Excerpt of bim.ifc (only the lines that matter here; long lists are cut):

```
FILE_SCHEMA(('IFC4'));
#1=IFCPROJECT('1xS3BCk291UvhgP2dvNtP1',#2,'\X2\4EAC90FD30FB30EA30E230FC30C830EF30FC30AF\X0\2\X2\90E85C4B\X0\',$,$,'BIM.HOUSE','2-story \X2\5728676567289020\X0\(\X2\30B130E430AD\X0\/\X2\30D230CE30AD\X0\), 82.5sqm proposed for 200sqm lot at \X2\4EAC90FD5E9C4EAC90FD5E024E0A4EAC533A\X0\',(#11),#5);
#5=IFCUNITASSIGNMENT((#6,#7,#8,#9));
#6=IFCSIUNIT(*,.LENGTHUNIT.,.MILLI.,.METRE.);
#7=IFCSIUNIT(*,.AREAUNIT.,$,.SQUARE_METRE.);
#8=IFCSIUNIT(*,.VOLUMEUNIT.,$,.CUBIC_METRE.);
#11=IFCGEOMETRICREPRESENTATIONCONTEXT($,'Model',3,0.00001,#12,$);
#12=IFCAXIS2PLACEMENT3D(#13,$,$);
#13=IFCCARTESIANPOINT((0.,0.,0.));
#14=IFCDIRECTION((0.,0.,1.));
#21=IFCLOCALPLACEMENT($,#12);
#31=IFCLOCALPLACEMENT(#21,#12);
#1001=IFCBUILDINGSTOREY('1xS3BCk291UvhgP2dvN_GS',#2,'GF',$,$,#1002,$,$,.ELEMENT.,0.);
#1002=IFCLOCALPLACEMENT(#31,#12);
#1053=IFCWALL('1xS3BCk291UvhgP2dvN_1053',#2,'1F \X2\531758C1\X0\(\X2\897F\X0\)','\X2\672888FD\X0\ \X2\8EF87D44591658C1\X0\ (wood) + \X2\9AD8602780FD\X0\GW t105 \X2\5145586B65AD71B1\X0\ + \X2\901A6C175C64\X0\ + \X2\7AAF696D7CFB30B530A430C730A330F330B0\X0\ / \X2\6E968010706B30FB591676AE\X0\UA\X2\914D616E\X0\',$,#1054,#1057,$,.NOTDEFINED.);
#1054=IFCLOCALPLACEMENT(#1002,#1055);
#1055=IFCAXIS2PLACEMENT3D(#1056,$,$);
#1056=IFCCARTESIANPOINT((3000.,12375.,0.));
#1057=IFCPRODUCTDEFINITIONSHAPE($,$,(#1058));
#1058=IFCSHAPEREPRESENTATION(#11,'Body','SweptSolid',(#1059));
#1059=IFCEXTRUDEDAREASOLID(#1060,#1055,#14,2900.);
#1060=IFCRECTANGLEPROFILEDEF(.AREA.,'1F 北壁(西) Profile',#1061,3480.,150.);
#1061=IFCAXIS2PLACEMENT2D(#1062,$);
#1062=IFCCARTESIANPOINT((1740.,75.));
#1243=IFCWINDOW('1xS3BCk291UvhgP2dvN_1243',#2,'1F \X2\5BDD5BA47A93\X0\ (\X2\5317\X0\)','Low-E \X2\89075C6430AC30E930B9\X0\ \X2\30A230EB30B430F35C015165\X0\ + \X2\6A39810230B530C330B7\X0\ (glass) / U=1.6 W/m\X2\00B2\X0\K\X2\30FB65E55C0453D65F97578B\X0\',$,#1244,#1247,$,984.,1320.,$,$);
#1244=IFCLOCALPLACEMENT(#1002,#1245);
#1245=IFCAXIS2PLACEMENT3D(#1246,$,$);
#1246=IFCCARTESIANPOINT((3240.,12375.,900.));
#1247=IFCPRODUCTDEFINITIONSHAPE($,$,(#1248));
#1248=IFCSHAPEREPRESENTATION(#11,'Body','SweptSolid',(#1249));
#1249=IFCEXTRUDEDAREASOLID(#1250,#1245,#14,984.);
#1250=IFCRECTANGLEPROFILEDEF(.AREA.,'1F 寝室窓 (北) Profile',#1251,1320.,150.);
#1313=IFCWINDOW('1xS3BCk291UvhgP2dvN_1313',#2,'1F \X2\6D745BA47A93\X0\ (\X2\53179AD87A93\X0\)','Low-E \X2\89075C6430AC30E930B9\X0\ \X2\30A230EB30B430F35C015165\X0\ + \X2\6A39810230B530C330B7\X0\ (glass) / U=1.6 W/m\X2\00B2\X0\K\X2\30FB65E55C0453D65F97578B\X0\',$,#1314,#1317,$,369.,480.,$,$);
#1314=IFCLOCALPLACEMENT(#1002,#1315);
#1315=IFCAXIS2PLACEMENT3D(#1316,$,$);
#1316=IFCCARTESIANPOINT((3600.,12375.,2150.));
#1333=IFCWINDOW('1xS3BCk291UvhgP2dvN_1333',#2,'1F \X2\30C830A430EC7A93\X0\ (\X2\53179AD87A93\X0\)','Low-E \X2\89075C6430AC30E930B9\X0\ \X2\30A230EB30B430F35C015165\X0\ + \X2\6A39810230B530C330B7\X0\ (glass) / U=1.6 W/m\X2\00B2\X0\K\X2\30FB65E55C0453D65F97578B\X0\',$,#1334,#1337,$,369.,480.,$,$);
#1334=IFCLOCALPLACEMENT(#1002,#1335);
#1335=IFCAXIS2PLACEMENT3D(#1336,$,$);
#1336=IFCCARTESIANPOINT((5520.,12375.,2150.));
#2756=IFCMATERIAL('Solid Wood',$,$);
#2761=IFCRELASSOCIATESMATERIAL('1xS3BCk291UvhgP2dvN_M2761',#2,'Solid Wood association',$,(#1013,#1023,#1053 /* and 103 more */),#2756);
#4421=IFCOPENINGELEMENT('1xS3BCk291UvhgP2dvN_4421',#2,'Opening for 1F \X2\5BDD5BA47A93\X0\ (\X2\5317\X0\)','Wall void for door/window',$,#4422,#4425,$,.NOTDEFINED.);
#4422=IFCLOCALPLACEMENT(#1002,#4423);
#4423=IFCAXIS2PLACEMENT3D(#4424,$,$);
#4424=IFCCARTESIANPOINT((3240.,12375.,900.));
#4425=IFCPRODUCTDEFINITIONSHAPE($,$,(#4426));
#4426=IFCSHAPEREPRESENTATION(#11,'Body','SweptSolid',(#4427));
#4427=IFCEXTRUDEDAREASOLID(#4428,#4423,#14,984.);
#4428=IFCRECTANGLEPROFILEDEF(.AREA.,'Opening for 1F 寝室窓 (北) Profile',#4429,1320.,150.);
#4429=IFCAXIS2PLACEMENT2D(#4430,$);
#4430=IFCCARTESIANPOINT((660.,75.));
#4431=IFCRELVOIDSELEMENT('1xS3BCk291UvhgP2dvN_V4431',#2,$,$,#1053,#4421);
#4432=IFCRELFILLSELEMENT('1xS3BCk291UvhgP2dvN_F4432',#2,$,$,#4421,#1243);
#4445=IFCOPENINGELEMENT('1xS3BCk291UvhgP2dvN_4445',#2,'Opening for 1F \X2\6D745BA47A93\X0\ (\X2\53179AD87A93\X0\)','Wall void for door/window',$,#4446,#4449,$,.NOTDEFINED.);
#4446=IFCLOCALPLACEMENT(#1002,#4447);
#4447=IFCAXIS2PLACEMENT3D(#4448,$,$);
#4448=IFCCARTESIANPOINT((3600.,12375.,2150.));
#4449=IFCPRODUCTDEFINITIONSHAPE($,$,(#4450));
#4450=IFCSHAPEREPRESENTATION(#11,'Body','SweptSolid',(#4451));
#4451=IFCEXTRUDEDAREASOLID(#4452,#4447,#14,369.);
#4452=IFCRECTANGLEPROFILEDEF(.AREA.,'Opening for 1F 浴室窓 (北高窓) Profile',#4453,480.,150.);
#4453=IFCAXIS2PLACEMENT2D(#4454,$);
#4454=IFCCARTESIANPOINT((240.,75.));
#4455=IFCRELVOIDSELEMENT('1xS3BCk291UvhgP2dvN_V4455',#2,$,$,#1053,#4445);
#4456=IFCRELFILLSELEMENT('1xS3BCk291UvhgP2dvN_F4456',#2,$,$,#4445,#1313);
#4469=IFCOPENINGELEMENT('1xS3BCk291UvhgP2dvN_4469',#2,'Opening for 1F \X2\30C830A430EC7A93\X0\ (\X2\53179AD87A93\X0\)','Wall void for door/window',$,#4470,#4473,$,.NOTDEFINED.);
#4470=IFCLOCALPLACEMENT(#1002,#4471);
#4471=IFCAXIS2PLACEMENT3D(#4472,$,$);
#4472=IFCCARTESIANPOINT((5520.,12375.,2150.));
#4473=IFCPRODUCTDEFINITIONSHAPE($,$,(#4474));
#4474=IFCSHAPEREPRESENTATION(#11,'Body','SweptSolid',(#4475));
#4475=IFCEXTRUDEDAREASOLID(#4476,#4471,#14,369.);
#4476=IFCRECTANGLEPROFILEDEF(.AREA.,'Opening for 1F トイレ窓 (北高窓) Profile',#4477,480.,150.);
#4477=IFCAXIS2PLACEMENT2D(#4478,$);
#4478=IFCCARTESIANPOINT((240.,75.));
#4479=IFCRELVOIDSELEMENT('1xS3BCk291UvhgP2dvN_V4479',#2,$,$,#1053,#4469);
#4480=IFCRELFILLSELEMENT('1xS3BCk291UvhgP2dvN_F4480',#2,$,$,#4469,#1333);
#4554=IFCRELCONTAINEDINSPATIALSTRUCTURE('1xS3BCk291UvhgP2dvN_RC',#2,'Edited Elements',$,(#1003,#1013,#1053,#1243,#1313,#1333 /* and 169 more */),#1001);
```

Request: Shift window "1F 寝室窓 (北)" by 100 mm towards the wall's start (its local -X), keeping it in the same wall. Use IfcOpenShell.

```python
import ifcopenshell
import ifcopenshell.api.geometry
import ifcopenshell.util.placement
import ifcopenshell.util.unit

model = ifcopenshell.open("bim.ifc")
unit_scale = ifcopenshell.util.unit.calculate_unit_scale(model)

window = model.by_id(1243)
opening = window.FillsVoids[0].RelatingOpeningElement
wall = opening.VoidsElements[0].RelatingBuildingElement

wall_matrix = ifcopenshell.util.placement.get_local_placement(wall.ObjectPlacement)
shift = wall_matrix[:3, 0] * -0.1 / unit_scale
before = ifcopenshell.util.placement.get_local_placement(window.ObjectPlacement)[:3, 3].copy()

# The window is not placed relative to its opening, so move both.
for product in (opening, window):
    matrix = ifcopenshell.util.placement.get_local_placement(product.ObjectPlacement)
    matrix[:3, 3] += shift
    ifcopenshell.api.geometry.edit_object_placement(model, product=product, matrix=matrix, is_si=False)

after = ifcopenshell.util.placement.get_local_placement(window.ObjectPlacement)[:3, 3]
print("window moved by", (after - before).round(3) + 0.0)

model.write("bim_rev.ifc")
```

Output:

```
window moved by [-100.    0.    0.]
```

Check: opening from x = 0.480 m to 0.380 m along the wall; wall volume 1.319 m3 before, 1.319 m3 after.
